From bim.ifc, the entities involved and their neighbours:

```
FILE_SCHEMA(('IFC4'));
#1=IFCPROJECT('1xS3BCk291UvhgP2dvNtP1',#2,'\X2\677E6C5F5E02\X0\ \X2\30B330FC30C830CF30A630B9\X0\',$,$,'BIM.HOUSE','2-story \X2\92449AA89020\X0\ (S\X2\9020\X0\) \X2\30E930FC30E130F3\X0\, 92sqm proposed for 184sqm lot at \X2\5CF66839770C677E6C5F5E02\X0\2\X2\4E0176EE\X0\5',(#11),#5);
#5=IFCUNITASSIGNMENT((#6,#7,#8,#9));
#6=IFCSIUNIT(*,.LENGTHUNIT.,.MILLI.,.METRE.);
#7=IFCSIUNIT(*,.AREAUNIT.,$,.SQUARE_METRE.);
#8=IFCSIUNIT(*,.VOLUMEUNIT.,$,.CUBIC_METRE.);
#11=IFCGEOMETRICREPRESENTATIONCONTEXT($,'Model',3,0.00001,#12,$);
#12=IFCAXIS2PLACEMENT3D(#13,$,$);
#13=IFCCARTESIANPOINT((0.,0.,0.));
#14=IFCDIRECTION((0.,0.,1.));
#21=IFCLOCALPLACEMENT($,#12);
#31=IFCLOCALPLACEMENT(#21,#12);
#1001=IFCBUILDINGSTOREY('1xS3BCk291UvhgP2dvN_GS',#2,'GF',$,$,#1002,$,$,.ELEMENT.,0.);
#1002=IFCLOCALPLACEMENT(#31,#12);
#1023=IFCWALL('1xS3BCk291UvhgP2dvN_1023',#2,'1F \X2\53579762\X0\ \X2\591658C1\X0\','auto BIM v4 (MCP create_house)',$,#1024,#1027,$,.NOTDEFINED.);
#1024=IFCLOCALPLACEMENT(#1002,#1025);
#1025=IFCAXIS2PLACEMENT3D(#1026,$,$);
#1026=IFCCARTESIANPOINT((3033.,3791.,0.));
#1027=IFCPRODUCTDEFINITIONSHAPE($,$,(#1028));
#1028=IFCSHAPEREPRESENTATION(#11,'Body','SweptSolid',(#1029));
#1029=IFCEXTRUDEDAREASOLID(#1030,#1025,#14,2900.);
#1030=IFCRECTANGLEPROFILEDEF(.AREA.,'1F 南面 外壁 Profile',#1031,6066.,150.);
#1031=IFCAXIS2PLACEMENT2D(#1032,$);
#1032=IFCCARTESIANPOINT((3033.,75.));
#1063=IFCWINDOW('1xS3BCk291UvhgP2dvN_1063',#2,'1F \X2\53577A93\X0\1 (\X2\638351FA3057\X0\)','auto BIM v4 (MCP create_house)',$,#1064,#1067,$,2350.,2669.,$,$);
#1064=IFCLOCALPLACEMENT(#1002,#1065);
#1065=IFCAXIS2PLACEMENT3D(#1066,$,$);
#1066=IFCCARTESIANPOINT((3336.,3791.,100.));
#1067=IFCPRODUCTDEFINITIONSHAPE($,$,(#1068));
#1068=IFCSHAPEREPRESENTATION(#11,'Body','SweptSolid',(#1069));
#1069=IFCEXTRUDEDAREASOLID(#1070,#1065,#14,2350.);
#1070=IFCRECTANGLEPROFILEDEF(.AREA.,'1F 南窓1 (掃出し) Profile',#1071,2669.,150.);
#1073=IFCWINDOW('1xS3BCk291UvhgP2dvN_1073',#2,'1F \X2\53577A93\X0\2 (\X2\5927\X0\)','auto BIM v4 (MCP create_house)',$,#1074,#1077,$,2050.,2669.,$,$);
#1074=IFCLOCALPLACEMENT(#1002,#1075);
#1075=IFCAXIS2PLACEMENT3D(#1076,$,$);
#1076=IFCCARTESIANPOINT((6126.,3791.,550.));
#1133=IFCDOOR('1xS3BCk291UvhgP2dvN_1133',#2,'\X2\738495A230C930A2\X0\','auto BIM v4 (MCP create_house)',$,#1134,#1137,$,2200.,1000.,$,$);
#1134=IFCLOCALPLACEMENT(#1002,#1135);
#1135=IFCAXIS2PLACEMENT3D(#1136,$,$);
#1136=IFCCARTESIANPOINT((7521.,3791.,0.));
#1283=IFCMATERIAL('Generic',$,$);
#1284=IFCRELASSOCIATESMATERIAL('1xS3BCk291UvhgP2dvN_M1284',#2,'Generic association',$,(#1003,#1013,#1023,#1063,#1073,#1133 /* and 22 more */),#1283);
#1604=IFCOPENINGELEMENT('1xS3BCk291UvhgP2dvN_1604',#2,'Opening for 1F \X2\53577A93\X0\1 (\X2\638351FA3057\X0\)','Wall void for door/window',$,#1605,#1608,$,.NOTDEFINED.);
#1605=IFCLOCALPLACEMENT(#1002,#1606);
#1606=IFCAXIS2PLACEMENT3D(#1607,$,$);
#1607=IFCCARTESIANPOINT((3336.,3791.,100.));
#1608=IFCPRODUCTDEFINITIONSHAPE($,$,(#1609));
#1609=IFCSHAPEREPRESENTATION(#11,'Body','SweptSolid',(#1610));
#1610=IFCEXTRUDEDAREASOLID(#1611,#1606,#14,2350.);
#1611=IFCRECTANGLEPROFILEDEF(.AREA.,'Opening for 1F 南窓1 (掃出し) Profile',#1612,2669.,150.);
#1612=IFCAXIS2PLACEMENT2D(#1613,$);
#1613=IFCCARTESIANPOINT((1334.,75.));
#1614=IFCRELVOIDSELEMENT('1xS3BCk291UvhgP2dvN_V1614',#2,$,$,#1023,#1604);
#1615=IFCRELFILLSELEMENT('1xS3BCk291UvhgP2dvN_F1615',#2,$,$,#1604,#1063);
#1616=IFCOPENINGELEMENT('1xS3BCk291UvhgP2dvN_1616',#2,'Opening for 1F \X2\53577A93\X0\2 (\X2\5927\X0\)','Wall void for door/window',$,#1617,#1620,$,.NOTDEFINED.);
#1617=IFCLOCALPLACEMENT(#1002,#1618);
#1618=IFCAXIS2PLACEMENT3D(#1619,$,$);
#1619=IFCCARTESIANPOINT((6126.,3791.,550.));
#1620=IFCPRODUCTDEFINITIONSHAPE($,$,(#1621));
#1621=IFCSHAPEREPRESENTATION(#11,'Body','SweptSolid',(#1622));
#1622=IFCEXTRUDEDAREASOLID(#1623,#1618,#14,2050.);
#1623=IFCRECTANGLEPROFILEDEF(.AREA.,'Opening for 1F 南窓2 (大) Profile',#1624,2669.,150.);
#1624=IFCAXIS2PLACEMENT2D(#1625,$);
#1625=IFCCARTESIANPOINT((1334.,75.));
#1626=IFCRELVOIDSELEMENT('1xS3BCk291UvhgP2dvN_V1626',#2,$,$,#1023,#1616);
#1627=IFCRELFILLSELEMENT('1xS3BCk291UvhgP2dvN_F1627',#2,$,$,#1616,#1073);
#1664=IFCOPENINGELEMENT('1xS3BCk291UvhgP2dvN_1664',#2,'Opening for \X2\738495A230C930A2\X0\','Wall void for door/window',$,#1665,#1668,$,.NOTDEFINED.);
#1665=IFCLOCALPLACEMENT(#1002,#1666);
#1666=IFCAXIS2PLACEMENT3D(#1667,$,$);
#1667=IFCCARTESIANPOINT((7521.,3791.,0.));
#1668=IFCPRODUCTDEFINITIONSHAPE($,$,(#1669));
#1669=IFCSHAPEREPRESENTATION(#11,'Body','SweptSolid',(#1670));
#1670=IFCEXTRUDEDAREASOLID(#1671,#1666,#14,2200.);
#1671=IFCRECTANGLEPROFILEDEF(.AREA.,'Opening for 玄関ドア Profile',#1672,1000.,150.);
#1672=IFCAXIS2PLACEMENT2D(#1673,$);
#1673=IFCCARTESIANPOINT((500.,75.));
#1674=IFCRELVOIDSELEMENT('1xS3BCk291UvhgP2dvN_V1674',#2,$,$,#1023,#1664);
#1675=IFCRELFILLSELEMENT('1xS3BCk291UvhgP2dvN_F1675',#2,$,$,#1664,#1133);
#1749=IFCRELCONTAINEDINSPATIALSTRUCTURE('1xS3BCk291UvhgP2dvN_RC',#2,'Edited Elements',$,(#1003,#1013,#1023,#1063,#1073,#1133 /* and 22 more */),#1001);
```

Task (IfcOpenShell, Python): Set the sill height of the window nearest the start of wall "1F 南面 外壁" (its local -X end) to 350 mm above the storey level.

```python
import numpy as np
import ifcopenshell
import ifcopenshell.api.geometry
import ifcopenshell.geom
import ifcopenshell.util.element
import ifcopenshell.util.placement
import ifcopenshell.util.shape
import ifcopenshell.util.unit

model = ifcopenshell.open("bim.ifc")
unit_scale = ifcopenshell.util.unit.calculate_unit_scale(model)

window = model.by_guid("1xS3BCk291UvhgP2dvN_1063")
opening = window.FillsVoids[0].RelatingOpeningElement
storey = ifcopenshell.util.element.get_container(window, ifc_class="IfcBuildingStorey")
level = ifcopenshell.util.placement.get_local_placement(storey.ObjectPlacement)[2, 3]

# The opening's origin need not be at the sill, so measure its lowest point.
shape = ifcopenshell.geom.create_shape(ifcopenshell.geom.settings(), opening)
bottom = ifcopenshell.util.shape.get_shape_bottom_elevation(shape, shape.geometry) / unit_scale
dz = level + 350.0 - bottom

shift = np.array([0.0, 0.0, dz])
# The window is not placed relative to its opening, so move both.
for product in (opening, window):
    matrix = ifcopenshell.util.placement.get_local_placement(product.ObjectPlacement)
    matrix[:3, 3] += shift
    ifcopenshell.api.geometry.edit_object_placement(model, product=product, matrix=matrix, is_si=False)

print(f"moved by {dz * unit_scale:+.3f} m")

model.write("bim_rev.ifc")
```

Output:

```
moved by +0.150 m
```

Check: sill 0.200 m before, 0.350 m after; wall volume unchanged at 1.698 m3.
